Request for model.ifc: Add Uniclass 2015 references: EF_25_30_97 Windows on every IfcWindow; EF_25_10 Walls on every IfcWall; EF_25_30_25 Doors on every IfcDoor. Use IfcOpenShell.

First a look at what the model holds.

```python
import ifcopenshell

model = ifcopenshell.open("model.ifc")
print(model.schema)
print("classifications:", [c.Name for c in model.by_type("IfcClassification")])
for ifc_class in ("IfcDoor", "IfcRoof", "IfcStair", "IfcWall", "IfcWindow"):
    print(ifc_class, len(model.by_type(ifc_class)))
```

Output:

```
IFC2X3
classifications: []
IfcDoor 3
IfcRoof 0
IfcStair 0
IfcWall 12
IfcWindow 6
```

```python
import ifcopenshell
import ifcopenshell.api.classification

model = ifcopenshell.open("model.ifc")

# IFC2X3 requires Source and Edition and has no link from the project to the system.
system = model.create_entity("IfcClassification", Source="NBS", Edition="2015", Name="Uniclass 2015")

codes = {
    "IfcWindow": ("EF_25_30_97", "Windows"),
    "IfcWall": ("EF_25_10", "Walls"),
    "IfcDoor": ("EF_25_30_25", "Doors"),
}
for ifc_class, (code, name) in codes.items():
    products = model.by_type(ifc_class)
    ifcopenshell.api.classification.add_reference(
        model, products=products, classification=system, identification=code, name=name
    )
    print(code, len(products))

model.write("model_edited.ifc")
```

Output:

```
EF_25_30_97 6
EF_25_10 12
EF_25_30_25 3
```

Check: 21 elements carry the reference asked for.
